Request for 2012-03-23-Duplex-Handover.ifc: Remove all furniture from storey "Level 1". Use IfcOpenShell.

First a look at what the model holds.

```python
import ifcopenshell
import ifcopenshell.util.element

model = ifcopenshell.open("2012-03-23-Duplex-Handover.ifc")
print(model.schema)
storey = next(s for s in model.by_type("IfcBuildingStorey") if s.Name == "Level 1")
furniture = [e for e in ifcopenshell.util.element.get_decomposition(storey) if e.is_a("IfcFurnishingElement")]
seen = {}
for e in furniture:
    element_type = ifcopenshell.util.element.get_type(e)
    name = element_type.Name if element_type not in (None, e) else None
    seen[name] = seen.get(name, 0) + 1
for name, count in sorted(seen.items(), key=str):
    print(count, "x", name)
```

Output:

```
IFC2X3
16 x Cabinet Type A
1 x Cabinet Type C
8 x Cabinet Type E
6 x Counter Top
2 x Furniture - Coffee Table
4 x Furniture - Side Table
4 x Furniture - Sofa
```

```python
import ifcopenshell
import ifcopenshell.api.root
import ifcopenshell.util.element

model = ifcopenshell.open("2012-03-23-Duplex-Handover.ifc")

storey = next(s for s in model.by_type("IfcBuildingStorey") if s.Name == "Level 1")
furniture = [e for e in ifcopenshell.util.element.get_decomposition(storey) if e.is_a("IfcFurnishingElement")]

for e in furniture:
    ifcopenshell.api.root.remove_product(model, product=e)
print(len(furniture), "removed")

model.write("2012-03-23-Duplex-Handover-out.ifc")
```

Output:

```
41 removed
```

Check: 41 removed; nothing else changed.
